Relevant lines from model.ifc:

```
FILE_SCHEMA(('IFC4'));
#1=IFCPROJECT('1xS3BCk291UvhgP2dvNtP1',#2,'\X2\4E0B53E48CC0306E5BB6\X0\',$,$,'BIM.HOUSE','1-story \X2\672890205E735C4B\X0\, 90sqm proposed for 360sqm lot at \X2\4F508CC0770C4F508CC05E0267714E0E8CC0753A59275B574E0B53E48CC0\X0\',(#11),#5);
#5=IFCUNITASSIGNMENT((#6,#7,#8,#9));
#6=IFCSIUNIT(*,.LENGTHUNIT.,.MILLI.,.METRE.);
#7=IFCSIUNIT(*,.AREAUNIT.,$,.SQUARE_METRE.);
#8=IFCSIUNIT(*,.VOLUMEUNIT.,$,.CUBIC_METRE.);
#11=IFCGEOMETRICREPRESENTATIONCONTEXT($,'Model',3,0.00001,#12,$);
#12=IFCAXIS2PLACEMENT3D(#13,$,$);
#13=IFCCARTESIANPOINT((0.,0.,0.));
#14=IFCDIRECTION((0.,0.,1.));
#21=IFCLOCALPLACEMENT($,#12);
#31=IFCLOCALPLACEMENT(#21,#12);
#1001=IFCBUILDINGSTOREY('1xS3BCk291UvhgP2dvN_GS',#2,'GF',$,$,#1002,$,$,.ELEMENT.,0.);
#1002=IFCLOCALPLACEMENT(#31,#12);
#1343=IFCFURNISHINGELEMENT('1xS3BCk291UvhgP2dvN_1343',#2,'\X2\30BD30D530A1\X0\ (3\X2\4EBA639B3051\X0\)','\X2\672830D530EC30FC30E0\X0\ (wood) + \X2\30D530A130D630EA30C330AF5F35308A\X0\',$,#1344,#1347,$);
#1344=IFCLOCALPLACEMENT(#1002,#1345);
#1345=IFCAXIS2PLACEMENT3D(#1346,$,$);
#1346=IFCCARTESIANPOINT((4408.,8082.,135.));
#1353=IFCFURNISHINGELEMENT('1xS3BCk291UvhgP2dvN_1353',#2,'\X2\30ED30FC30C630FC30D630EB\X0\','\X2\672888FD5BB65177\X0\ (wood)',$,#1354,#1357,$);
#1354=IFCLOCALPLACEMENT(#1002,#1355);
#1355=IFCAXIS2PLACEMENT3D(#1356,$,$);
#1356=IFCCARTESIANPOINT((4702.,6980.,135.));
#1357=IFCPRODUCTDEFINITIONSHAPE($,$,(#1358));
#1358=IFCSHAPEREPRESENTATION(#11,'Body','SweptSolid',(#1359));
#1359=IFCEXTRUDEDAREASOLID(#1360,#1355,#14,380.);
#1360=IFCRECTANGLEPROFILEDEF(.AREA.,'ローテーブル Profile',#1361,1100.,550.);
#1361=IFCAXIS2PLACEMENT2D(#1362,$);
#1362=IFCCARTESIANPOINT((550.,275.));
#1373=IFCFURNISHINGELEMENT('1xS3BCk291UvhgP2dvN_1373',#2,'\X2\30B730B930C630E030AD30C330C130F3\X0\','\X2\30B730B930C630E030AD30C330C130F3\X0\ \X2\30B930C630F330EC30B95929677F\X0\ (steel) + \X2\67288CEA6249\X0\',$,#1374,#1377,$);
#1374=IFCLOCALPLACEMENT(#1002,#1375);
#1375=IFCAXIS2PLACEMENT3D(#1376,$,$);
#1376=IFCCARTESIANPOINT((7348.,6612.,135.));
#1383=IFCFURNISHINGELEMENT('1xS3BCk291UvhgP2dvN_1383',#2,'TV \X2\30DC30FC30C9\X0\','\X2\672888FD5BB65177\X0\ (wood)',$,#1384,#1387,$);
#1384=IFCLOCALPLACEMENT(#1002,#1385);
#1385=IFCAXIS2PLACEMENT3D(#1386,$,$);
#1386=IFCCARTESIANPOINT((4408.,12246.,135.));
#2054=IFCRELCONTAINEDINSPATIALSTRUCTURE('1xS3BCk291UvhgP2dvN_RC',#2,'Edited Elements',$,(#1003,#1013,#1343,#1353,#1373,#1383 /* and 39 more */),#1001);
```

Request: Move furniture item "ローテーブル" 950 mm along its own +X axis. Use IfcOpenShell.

```python
import ifcopenshell
import ifcopenshell.api.geometry
import ifcopenshell.util.placement
import ifcopenshell.util.unit

model = ifcopenshell.open("model.ifc")
unit_scale = ifcopenshell.util.unit.calculate_unit_scale(model)

item = model.by_guid("1xS3BCk291UvhgP2dvN_1353")
matrix = ifcopenshell.util.placement.get_local_placement(item.ObjectPlacement)
matrix[:3, 3] += matrix[:3, 0] * 0.95 / unit_scale
ifcopenshell.api.geometry.edit_object_placement(model, product=item, matrix=matrix, is_si=False)

print(ifcopenshell.util.placement.get_local_placement(item.ObjectPlacement).round(3) + 0.0)

model.write("model_edited.ifc")
```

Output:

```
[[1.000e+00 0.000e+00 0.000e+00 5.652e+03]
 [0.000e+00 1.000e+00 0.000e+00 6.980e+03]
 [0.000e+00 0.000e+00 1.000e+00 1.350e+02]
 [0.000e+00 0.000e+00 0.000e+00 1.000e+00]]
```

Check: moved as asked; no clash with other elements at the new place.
